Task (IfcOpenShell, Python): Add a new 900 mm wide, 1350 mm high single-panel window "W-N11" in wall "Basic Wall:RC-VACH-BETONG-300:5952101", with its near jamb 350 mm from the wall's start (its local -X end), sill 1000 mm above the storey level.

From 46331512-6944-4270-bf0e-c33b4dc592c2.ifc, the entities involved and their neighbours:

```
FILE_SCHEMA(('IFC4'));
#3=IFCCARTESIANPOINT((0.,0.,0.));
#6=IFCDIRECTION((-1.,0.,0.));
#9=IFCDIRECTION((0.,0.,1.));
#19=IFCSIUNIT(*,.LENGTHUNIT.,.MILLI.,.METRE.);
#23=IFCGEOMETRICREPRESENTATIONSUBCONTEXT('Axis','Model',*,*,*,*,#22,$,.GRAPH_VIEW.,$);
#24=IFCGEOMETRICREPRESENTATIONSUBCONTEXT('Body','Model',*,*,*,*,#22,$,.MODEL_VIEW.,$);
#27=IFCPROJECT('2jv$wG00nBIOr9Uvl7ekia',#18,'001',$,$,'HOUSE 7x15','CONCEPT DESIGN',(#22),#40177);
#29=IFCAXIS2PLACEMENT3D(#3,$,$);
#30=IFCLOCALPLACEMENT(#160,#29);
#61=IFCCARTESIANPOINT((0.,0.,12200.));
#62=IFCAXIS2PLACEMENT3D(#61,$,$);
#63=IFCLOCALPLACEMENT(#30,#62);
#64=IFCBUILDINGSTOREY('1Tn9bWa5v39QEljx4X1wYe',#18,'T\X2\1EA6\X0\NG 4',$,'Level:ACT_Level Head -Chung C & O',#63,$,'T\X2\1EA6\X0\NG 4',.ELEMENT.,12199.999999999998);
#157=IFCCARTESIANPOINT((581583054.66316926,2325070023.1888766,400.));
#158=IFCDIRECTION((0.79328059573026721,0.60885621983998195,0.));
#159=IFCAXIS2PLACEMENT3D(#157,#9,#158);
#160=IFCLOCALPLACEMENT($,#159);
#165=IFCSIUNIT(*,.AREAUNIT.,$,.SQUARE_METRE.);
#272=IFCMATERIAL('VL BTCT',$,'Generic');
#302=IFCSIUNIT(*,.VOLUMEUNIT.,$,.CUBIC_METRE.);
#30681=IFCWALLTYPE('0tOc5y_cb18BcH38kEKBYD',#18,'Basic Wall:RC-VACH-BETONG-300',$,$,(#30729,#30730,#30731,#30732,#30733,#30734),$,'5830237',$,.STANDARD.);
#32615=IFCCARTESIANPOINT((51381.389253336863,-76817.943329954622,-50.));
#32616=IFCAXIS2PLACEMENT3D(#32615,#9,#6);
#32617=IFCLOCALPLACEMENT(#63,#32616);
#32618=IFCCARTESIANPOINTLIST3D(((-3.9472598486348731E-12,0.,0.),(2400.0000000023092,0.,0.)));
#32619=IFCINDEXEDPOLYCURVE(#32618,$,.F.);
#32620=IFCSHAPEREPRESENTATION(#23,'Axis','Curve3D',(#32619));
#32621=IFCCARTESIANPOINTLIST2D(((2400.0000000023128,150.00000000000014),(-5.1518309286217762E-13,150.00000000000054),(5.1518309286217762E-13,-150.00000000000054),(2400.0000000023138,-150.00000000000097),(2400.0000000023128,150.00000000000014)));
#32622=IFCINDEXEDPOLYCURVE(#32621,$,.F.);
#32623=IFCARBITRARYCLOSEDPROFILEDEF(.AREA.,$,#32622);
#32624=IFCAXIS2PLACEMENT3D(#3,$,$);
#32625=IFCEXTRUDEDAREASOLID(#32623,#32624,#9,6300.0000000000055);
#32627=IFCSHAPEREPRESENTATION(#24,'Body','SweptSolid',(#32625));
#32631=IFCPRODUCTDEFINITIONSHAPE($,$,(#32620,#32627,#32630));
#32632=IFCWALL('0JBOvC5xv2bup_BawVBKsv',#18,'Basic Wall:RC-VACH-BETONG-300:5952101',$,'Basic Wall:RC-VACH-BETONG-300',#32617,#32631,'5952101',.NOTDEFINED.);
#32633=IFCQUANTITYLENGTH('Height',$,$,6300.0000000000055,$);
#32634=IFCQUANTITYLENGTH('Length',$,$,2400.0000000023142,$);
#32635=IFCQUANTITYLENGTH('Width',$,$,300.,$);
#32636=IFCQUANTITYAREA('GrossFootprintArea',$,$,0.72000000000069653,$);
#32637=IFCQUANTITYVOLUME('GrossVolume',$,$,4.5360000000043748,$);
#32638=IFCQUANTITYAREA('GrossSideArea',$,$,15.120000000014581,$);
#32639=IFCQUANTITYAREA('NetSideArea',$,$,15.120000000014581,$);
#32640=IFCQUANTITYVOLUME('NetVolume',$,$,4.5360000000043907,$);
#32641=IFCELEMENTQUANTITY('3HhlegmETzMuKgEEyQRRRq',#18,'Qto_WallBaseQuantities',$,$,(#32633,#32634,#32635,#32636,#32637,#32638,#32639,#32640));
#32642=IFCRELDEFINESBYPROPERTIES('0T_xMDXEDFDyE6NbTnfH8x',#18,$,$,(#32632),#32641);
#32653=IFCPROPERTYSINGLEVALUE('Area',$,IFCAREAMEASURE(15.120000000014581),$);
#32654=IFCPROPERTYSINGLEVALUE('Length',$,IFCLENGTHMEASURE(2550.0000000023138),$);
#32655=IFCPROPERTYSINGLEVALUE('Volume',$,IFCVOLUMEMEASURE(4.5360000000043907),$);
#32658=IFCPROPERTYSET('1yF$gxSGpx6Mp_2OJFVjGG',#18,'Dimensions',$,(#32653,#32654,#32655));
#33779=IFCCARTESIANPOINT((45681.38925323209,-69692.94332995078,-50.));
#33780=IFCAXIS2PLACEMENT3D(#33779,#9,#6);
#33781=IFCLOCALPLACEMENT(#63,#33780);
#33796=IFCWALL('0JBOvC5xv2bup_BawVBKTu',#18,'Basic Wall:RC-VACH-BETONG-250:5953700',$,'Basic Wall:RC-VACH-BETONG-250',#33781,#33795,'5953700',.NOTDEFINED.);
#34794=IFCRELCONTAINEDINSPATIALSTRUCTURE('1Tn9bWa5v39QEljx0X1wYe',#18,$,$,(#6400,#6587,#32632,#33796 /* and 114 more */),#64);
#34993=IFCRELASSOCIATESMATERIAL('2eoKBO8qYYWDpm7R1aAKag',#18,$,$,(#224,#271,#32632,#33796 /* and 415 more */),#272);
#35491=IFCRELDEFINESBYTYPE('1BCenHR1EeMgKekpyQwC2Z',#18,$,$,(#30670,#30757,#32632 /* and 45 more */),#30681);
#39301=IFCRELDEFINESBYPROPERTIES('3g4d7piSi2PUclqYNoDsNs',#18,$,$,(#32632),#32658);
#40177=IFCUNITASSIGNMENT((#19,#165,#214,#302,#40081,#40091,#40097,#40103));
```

```python
import numpy as np
import ifcopenshell
import ifcopenshell.api.feature
import ifcopenshell.api.geometry
import ifcopenshell.api.pset
import ifcopenshell.api.root
import ifcopenshell.api.spatial
import ifcopenshell.geom
import ifcopenshell.util.element
import ifcopenshell.util.placement
import ifcopenshell.util.representation
import ifcopenshell.util.shape
import ifcopenshell.util.unit

model = ifcopenshell.open("46331512-6944-4270-bf0e-c33b4dc592c2.ifc")
unit_scale = ifcopenshell.util.unit.calculate_unit_scale(model)
area_scale = ifcopenshell.util.unit.calculate_unit_scale(model, "AREAUNIT")
volume_scale = ifcopenshell.util.unit.calculate_unit_scale(model, "VOLUMEUNIT")
settings = ifcopenshell.geom.settings()


def volume(element):
    """Net volume in cubic metres, openings subtracted."""
    shape = ifcopenshell.geom.create_shape(settings, element)
    return ifcopenshell.util.shape.get_volume(shape.geometry)


wall = model.by_id(32632)
storey = ifcopenshell.util.element.get_container(wall, ifc_class="IfcBuildingStorey")
context = ifcopenshell.util.representation.get_context(model, "Model", "Body", "MODEL_VIEW")
before = volume(wall)

width, height, from_end, sill = 0.9, 1.35, 0.35, 1  # metres

# The wall runs along its own X axis, and the end named is its -X end.
wall_shape = ifcopenshell.geom.create_shape(settings, wall)
x, y, z = ifcopenshell.util.shape.get_vertices(wall_shape.geometry).T
start = x.min() + from_end
face, thickness = float(y.min()), float(y.max() - y.min())
wall_matrix = ifcopenshell.util.placement.get_local_placement(wall.ObjectPlacement)
level = ifcopenshell.util.placement.get_local_placement(storey.ObjectPlacement)[2, 3]


def in_wall(x, y):
    """Placement at x, y metres in the wall's axes, at sill height."""
    matrix = wall_matrix.copy()
    matrix[:, 3] = wall_matrix @ np.array([x / unit_scale, y / unit_scale, 0.0, 1.0])
    matrix[2, 3] = level + sill / unit_scale
    return matrix


# Opening: a box that overshoots both wall faces by 50 mm.
opening = ifcopenshell.api.root.create_entity(model, ifc_class="IfcOpeningElement", predefined_type="OPENING")
box = ifcopenshell.api.geometry.add_wall_representation(
    model, context=context, length=width, height=height, thickness=thickness + 0.1
)
ifcopenshell.api.geometry.assign_representation(model, product=opening, representation=box)
ifcopenshell.api.geometry.edit_object_placement(model, product=opening, matrix=in_wall(start, face - 0.05), is_si=False)
ifcopenshell.api.feature.add_feature(model, feature=opening, element=wall)

window = ifcopenshell.api.root.create_entity(model, ifc_class="IfcWindow", name="W-N11", predefined_type="WINDOW")
window.OverallWidth, window.OverallHeight = width / unit_scale, height / unit_scale
window.PartitioningType = "SINGLE_PANEL"
body = ifcopenshell.api.geometry.add_window_representation(
    model,
    context=context,
    overall_width=window.OverallWidth,
    overall_height=window.OverallHeight,
    partition_type="SINGLE_PANEL",
)
ifcopenshell.api.geometry.assign_representation(model, product=window, representation=body)
ifcopenshell.api.spatial.assign_container(model, products=[window], relating_structure=storey)
ifcopenshell.api.feature.add_filling(model, opening=opening, element=window)

# Centre the window in the wall's thickness.
ifcopenshell.api.geometry.edit_object_placement(model, product=window, matrix=in_wall(start, face), is_si=False)
window_shape = ifcopenshell.geom.create_shape(settings, window)
depth = ifcopenshell.util.shape.get_vertices(window_shape.geometry)[:, 1]
offset = face + thickness / 2 - (depth.min() + depth.max()) / 2
ifcopenshell.api.geometry.edit_object_placement(model, product=window, matrix=in_wall(start, offset), is_si=False)

after = volume(wall)

# Update the wall's stored quantities.
qto = model.by_id(ifcopenshell.util.element.get_pset(wall, "Qto_WallBaseQuantities", should_inherit=False)["id"])
ifcopenshell.api.pset.edit_qto(model, qto=qto, properties={
    "NetSideArea": after / thickness / area_scale,
    "NetVolume": after / volume_scale,
})
pset = model.by_id(ifcopenshell.util.element.get_pset(wall, "Dimensions", should_inherit=False)["id"])
ifcopenshell.api.pset.edit_pset(model, pset=pset, properties={
    "Area": model.create_entity("IfcAreaMeasure", after / thickness / area_scale),
    "Volume": model.create_entity("IfcVolumeMeasure", after / volume_scale),
})

print(f"wall volume {before:.3f} -> {after:.3f} m3")

model.write("46331512-6944-4270-bf0e-c33b4dc592c2_updated.ifc")
```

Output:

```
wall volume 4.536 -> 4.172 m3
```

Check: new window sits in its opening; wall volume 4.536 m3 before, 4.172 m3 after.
